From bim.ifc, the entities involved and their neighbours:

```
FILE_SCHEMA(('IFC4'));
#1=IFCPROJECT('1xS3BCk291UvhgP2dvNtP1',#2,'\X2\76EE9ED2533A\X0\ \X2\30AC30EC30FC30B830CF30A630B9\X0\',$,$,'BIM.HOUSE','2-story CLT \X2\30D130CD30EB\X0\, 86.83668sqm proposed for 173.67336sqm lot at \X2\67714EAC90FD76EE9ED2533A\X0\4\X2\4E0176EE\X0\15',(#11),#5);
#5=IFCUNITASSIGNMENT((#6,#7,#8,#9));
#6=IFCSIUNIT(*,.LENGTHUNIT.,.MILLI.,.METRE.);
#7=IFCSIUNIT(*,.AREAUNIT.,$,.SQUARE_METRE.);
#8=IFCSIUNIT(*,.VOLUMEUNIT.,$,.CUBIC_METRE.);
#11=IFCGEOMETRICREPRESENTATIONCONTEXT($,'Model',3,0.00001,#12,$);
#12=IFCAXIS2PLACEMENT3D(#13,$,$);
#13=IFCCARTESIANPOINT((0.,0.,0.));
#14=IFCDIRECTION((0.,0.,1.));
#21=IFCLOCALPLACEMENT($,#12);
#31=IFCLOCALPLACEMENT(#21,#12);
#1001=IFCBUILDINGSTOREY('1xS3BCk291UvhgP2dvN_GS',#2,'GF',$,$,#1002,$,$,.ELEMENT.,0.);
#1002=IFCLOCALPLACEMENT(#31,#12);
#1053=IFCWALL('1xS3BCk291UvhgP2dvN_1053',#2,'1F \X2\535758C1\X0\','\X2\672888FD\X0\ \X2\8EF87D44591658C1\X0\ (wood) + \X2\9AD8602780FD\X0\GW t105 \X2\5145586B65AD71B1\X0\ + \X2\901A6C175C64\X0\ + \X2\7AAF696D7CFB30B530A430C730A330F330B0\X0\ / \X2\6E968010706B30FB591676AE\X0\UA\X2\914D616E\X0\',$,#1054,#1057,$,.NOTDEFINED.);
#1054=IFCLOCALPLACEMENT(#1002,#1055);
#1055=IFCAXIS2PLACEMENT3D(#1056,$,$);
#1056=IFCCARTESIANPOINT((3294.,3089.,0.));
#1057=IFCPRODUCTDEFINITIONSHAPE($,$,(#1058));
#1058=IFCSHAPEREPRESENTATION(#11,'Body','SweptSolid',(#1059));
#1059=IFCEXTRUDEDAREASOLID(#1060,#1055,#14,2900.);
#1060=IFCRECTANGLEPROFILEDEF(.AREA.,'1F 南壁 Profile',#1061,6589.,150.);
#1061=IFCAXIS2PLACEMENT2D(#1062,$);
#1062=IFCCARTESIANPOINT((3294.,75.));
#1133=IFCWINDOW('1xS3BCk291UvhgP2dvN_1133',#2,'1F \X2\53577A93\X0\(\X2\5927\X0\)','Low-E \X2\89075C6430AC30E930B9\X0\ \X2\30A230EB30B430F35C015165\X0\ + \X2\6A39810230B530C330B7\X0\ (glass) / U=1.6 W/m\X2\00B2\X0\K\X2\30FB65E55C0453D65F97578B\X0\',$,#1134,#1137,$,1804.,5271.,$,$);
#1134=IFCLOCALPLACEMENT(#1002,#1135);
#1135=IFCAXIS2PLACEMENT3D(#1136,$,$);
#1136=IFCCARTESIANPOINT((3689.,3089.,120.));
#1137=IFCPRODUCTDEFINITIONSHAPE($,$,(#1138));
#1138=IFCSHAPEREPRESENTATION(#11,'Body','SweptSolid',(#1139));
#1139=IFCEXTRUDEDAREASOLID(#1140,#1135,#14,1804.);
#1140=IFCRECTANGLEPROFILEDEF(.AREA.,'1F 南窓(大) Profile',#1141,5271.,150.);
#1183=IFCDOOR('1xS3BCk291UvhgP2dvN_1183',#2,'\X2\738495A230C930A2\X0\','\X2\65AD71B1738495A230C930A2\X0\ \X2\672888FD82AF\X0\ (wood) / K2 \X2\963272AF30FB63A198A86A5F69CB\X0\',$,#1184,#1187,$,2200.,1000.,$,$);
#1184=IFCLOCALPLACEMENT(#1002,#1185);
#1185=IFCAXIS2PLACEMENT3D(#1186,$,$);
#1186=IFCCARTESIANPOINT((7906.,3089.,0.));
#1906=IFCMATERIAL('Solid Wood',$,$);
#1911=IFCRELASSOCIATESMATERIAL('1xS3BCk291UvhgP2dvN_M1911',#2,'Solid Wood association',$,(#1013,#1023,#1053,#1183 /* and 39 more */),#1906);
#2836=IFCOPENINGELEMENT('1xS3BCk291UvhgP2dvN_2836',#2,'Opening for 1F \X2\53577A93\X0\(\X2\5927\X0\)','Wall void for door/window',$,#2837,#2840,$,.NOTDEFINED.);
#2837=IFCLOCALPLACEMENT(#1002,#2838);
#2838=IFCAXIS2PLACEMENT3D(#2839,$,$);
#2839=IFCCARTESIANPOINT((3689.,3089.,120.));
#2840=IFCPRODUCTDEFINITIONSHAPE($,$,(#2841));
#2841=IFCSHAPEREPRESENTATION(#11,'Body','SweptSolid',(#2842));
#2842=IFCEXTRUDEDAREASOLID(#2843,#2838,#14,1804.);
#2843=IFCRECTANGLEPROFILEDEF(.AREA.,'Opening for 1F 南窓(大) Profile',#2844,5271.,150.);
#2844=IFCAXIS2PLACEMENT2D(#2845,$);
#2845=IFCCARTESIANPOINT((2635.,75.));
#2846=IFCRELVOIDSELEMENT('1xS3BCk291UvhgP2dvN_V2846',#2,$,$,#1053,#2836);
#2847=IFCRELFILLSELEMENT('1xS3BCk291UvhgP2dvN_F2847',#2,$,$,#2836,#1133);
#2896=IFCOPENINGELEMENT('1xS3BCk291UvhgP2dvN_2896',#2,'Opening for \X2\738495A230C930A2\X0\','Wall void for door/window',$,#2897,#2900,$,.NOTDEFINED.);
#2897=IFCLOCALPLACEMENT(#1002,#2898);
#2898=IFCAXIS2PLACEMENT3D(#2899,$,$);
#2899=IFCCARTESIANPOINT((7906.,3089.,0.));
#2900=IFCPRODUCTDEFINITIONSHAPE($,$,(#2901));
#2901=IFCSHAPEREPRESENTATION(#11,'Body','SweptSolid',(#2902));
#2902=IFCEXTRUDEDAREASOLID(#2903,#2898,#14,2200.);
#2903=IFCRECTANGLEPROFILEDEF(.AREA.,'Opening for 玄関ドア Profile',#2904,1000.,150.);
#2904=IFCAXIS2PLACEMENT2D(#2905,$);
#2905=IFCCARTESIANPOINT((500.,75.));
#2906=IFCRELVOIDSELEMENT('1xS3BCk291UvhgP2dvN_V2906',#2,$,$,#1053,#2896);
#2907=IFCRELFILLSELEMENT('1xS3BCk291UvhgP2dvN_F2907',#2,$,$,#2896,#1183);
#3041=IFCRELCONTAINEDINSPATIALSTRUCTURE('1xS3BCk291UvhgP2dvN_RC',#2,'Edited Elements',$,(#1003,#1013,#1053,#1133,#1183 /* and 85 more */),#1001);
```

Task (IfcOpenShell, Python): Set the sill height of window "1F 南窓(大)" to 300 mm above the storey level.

```python
import numpy as np
import ifcopenshell
import ifcopenshell.api.geometry
import ifcopenshell.geom
import ifcopenshell.util.element
import ifcopenshell.util.placement
import ifcopenshell.util.shape
import ifcopenshell.util.unit

model = ifcopenshell.open("bim.ifc")
unit_scale = ifcopenshell.util.unit.calculate_unit_scale(model)

window = model.by_id(1133)
opening = window.FillsVoids[0].RelatingOpeningElement
storey = ifcopenshell.util.element.get_container(window, ifc_class="IfcBuildingStorey")
level = ifcopenshell.util.placement.get_local_placement(storey.ObjectPlacement)[2, 3]

# The opening's origin need not be at the sill, so measure its lowest point.
shape = ifcopenshell.geom.create_shape(ifcopenshell.geom.settings(), opening)
bottom = ifcopenshell.util.shape.get_shape_bottom_elevation(shape, shape.geometry) / unit_scale
dz = level + 0.3 / unit_scale - bottom

shift = np.array([0.0, 0.0, dz])
# The window is not placed relative to its opening, so move both.
for product in (opening, window):
    matrix = ifcopenshell.util.placement.get_local_placement(product.ObjectPlacement)
    matrix[:3, 3] += shift
    ifcopenshell.api.geometry.edit_object_placement(model, product=product, matrix=matrix, is_si=False)

print(f"moved by {dz * unit_scale:+.3f} m")

model.write("bim_updated.ifc")
```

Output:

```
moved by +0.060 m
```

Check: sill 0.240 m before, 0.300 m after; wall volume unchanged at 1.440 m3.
